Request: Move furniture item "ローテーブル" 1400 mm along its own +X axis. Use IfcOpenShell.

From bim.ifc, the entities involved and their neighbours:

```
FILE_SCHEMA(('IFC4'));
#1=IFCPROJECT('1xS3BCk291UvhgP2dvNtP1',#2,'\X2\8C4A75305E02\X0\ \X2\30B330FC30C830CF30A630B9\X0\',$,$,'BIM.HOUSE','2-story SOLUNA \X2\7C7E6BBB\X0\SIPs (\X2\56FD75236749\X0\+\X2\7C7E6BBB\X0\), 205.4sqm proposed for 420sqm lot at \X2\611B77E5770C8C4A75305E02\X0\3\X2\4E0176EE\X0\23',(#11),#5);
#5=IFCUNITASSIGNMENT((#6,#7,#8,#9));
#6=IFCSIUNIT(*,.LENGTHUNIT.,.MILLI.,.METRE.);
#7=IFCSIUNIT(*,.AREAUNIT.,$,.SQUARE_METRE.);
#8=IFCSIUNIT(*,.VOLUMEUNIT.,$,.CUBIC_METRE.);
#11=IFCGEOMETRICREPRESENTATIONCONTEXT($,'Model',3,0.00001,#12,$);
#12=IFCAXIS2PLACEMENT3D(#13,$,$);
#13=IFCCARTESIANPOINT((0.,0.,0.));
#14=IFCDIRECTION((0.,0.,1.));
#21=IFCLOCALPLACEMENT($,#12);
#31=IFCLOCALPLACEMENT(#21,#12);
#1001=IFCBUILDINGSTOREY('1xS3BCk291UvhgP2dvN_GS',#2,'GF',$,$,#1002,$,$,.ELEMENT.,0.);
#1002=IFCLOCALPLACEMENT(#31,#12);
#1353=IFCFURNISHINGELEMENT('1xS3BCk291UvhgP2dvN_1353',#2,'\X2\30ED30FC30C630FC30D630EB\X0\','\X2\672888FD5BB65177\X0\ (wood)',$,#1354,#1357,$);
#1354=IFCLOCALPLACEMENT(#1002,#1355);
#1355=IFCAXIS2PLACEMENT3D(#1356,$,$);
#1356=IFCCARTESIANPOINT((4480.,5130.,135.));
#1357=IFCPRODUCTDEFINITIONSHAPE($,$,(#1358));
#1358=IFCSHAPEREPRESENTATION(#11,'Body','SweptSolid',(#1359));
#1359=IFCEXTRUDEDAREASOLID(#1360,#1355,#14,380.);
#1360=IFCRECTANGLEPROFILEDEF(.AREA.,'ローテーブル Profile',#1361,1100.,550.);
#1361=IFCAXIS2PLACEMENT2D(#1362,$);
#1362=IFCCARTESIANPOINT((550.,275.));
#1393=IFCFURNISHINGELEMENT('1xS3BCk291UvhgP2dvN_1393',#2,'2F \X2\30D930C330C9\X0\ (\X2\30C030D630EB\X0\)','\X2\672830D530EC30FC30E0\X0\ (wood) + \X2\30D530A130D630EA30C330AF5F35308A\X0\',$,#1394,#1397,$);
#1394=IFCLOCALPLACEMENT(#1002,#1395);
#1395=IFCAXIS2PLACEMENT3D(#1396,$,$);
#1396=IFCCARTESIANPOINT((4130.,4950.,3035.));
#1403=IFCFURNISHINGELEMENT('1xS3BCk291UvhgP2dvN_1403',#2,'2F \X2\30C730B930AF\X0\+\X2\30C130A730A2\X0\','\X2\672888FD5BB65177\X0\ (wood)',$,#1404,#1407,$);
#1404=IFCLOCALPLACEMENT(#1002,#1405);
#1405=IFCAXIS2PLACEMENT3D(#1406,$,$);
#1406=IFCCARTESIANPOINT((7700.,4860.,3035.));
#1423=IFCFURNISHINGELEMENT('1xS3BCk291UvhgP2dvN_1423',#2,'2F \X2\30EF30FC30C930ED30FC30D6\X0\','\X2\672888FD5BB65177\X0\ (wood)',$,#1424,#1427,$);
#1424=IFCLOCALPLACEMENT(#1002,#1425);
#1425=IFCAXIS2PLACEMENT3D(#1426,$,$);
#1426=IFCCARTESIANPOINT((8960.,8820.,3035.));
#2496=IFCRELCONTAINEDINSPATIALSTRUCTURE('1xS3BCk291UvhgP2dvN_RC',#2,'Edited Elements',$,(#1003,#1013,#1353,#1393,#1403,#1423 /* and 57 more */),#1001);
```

```python
import ifcopenshell
import ifcopenshell.api.geometry
import ifcopenshell.util.placement

model = ifcopenshell.open("bim.ifc")

item = model.by_guid("1xS3BCk291UvhgP2dvN_1353")
matrix = ifcopenshell.util.placement.get_local_placement(item.ObjectPlacement)
matrix[:3, 3] += matrix[:3, 0] * 1400.0
ifcopenshell.api.geometry.edit_object_placement(model, product=item, matrix=matrix, is_si=False)

print(ifcopenshell.util.placement.get_local_placement(item.ObjectPlacement).round(3) + 0.0)

model.write("bim_edited.ifc")
```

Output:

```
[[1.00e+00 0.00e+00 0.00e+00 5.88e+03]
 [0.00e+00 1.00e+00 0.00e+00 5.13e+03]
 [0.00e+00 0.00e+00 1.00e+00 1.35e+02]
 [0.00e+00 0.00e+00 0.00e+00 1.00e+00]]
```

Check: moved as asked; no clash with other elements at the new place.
